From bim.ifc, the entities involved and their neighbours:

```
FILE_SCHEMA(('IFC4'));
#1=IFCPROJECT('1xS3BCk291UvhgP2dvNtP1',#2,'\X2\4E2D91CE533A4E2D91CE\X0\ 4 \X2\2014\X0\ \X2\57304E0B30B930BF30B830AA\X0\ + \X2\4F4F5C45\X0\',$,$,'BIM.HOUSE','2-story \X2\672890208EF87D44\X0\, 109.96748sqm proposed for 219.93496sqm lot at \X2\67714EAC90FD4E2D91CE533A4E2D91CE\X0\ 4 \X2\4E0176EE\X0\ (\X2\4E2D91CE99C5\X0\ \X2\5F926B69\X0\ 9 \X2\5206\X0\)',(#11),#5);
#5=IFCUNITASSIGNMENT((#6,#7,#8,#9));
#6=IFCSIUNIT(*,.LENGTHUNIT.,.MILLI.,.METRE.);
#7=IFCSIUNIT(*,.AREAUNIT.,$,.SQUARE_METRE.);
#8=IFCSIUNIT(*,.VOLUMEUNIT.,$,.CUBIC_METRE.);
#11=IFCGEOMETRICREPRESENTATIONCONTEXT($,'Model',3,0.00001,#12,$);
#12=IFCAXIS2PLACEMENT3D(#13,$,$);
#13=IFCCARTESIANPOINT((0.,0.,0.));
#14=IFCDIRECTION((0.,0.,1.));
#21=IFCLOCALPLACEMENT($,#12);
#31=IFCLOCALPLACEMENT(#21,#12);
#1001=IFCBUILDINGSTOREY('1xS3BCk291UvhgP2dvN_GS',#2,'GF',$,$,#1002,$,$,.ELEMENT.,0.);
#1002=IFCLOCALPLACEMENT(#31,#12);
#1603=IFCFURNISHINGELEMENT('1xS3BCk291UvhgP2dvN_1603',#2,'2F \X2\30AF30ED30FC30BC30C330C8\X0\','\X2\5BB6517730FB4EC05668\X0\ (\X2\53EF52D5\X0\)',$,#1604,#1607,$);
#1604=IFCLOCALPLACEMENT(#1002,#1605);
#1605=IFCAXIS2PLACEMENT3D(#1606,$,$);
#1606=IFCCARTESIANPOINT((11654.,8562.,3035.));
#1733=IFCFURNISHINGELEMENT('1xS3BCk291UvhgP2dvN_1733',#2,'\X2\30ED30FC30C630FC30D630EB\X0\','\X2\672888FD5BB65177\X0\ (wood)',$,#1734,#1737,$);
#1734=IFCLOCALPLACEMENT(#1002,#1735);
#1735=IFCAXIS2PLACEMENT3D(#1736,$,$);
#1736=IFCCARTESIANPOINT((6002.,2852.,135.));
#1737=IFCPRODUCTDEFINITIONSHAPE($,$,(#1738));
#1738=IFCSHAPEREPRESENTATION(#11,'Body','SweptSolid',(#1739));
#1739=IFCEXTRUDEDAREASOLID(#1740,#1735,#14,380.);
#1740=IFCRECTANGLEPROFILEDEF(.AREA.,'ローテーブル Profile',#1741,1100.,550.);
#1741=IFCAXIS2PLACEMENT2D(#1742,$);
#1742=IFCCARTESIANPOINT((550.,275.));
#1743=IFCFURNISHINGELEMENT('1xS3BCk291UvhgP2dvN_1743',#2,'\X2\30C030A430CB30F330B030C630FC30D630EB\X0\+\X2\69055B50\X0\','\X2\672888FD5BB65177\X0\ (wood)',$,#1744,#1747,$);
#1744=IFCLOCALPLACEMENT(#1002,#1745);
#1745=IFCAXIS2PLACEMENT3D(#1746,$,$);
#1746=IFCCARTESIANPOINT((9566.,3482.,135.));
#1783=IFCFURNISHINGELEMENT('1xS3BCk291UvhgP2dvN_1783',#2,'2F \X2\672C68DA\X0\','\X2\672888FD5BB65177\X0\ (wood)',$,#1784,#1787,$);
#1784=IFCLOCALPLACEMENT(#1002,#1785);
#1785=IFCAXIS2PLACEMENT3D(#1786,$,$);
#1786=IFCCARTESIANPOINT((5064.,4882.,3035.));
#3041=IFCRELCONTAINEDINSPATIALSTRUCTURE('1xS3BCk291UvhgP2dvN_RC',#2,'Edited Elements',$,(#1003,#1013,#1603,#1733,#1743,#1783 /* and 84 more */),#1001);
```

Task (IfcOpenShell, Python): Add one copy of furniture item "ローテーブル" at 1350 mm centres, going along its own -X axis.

```python
import ifcopenshell
import ifcopenshell.api.geometry
import ifcopenshell.api.root
import ifcopenshell.util.element
import ifcopenshell.util.placement
import ifcopenshell.util.unit

model = ifcopenshell.open("bim.ifc")
unit_scale = ifcopenshell.util.unit.calculate_unit_scale(model)


def reuse_history(source, copy):
    """copy_class also copies each property set's owner history, people and application; keep the originals."""
    for rel in copy.IsDefinedBy:
        if rel.is_a("IfcRelDefinesByProperties") and (history := rel.RelatingPropertyDefinition.OwnerHistory):
            rel.RelatingPropertyDefinition.OwnerHistory = source.OwnerHistory
            ifcopenshell.util.element.remove_deep2(model, history)


source = model.by_id(1733)
base = ifcopenshell.util.placement.get_local_placement(source.ObjectPlacement)
step = -base[:3, 0] * 1.35 / unit_scale

for i in range(1, 2):
    copy = ifcopenshell.api.root.copy_class(model, product=source)
    copy.Representation = ifcopenshell.util.element.copy_deep(
        model, source.Representation, exclude=["IfcGeometricRepresentationContext", "IfcRepresentationMap"]
    )
    reuse_history(source, copy)
    matrix = base.copy()
    matrix[:3, 3] += i * step
    print("added at", matrix[:3, 3].round(3) + 0.0)
    ifcopenshell.api.geometry.edit_object_placement(model, product=copy, matrix=matrix, is_si=False)

model.write("bim_edited.ifc")
```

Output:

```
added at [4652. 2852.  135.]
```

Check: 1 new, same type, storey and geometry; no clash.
